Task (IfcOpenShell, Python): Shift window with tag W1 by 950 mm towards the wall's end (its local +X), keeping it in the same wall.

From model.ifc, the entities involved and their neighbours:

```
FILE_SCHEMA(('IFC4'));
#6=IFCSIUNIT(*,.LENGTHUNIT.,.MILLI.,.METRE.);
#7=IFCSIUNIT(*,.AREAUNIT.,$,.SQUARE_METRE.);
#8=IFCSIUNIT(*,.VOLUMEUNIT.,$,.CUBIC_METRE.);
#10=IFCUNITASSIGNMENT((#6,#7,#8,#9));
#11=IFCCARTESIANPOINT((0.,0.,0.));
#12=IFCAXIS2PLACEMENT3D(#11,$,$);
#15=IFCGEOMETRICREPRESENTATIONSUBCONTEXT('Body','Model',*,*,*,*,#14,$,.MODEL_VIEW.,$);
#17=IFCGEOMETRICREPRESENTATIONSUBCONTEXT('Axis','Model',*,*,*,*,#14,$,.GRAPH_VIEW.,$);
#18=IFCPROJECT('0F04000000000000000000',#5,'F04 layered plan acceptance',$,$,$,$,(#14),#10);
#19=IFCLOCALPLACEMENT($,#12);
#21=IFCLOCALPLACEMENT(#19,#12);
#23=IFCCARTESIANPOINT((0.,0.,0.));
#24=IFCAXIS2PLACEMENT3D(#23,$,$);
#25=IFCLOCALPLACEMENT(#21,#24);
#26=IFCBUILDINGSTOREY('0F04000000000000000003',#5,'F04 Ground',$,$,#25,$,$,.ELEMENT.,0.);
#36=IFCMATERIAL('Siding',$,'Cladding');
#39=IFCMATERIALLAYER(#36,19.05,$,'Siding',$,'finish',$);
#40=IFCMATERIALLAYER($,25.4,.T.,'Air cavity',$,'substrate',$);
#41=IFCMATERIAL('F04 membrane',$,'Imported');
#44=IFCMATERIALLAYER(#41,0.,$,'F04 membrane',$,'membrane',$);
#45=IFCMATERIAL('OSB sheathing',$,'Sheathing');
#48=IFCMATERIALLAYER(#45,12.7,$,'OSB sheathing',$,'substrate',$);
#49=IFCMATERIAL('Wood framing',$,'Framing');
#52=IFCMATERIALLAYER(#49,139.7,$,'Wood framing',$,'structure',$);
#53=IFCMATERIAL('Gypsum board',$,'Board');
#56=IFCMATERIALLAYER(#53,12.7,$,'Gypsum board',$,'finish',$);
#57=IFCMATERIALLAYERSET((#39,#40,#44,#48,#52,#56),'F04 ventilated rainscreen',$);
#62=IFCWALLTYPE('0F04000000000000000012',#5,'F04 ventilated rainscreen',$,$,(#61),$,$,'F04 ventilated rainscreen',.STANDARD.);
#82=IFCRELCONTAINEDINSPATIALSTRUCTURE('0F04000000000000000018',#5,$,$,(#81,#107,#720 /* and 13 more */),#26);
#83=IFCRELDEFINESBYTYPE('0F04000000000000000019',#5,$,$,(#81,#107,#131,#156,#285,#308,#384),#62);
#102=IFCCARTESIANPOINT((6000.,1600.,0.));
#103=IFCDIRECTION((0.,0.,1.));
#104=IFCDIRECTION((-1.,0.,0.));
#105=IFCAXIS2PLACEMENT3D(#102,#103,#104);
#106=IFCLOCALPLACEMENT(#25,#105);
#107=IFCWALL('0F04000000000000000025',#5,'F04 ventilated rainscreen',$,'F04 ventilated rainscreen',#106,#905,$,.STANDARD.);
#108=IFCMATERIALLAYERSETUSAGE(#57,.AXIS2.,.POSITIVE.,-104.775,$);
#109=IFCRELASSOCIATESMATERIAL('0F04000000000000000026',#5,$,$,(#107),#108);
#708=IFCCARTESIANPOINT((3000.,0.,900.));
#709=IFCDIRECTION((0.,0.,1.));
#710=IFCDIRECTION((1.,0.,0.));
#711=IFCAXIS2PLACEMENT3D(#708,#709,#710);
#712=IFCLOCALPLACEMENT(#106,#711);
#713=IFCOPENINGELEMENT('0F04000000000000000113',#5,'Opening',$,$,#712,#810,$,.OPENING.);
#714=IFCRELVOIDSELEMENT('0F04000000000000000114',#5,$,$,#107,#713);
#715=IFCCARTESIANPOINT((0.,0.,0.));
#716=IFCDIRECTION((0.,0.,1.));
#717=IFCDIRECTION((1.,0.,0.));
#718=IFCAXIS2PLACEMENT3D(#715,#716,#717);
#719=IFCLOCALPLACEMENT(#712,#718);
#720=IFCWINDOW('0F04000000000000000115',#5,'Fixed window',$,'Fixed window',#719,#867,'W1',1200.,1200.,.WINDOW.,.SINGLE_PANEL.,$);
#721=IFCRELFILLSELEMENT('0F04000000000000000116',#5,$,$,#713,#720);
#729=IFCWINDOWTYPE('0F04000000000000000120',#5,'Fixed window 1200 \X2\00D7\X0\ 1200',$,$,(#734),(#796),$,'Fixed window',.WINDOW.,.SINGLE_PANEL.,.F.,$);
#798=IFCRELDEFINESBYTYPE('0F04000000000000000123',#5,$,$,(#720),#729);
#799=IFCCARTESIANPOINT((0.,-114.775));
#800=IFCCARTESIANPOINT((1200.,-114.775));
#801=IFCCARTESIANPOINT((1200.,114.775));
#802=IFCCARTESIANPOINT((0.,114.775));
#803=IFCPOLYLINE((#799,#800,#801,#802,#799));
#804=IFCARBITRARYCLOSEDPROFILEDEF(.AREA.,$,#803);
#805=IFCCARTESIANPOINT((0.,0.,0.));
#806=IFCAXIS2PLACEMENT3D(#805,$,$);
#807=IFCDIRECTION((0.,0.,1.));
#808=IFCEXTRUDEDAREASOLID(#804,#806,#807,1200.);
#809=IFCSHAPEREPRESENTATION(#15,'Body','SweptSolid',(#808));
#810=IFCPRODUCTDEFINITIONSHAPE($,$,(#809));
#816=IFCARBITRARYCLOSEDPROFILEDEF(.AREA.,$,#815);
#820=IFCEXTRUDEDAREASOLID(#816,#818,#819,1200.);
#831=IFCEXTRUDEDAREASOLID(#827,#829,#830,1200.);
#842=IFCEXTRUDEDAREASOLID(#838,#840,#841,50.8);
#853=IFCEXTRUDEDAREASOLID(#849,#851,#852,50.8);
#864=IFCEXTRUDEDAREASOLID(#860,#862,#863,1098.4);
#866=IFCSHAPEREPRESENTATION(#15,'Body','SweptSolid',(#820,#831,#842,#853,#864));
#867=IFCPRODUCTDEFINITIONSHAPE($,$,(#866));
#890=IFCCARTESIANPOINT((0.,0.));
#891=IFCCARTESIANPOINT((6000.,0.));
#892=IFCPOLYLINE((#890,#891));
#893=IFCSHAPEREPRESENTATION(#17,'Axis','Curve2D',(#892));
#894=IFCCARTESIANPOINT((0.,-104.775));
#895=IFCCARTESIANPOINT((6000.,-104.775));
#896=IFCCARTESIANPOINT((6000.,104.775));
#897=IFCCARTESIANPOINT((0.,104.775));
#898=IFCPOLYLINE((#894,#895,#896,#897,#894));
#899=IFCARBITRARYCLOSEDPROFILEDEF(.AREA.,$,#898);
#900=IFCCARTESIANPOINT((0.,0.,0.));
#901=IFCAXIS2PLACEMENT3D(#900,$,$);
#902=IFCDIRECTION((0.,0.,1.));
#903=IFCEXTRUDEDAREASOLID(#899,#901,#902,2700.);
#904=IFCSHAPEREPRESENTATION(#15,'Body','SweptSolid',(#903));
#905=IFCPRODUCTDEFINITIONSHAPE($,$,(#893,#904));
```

```python
import ifcopenshell
import ifcopenshell.api.geometry
import ifcopenshell.util.placement

model = ifcopenshell.open("model.ifc")

window = model.by_id(720)
opening = window.FillsVoids[0].RelatingOpeningElement
wall = opening.VoidsElements[0].RelatingBuildingElement

wall_matrix = ifcopenshell.util.placement.get_local_placement(wall.ObjectPlacement)
shift = wall_matrix[:3, 0] * 950.0
before = ifcopenshell.util.placement.get_local_placement(window.ObjectPlacement)[:3, 3].copy()

# The window is placed relative to its opening, so it follows when the opening moves.
matrix = ifcopenshell.util.placement.get_local_placement(opening.ObjectPlacement)
matrix[:3, 3] += shift
ifcopenshell.api.geometry.edit_object_placement(
    model, product=opening, matrix=matrix, is_si=False, should_transform_children=True
)

after = ifcopenshell.util.placement.get_local_placement(window.ObjectPlacement)[:3, 3]
print("window moved by", (after - before).round(3) + 0.0)

model.write("model_updated.ifc")
```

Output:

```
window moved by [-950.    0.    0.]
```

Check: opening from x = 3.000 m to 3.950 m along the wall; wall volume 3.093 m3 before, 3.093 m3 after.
